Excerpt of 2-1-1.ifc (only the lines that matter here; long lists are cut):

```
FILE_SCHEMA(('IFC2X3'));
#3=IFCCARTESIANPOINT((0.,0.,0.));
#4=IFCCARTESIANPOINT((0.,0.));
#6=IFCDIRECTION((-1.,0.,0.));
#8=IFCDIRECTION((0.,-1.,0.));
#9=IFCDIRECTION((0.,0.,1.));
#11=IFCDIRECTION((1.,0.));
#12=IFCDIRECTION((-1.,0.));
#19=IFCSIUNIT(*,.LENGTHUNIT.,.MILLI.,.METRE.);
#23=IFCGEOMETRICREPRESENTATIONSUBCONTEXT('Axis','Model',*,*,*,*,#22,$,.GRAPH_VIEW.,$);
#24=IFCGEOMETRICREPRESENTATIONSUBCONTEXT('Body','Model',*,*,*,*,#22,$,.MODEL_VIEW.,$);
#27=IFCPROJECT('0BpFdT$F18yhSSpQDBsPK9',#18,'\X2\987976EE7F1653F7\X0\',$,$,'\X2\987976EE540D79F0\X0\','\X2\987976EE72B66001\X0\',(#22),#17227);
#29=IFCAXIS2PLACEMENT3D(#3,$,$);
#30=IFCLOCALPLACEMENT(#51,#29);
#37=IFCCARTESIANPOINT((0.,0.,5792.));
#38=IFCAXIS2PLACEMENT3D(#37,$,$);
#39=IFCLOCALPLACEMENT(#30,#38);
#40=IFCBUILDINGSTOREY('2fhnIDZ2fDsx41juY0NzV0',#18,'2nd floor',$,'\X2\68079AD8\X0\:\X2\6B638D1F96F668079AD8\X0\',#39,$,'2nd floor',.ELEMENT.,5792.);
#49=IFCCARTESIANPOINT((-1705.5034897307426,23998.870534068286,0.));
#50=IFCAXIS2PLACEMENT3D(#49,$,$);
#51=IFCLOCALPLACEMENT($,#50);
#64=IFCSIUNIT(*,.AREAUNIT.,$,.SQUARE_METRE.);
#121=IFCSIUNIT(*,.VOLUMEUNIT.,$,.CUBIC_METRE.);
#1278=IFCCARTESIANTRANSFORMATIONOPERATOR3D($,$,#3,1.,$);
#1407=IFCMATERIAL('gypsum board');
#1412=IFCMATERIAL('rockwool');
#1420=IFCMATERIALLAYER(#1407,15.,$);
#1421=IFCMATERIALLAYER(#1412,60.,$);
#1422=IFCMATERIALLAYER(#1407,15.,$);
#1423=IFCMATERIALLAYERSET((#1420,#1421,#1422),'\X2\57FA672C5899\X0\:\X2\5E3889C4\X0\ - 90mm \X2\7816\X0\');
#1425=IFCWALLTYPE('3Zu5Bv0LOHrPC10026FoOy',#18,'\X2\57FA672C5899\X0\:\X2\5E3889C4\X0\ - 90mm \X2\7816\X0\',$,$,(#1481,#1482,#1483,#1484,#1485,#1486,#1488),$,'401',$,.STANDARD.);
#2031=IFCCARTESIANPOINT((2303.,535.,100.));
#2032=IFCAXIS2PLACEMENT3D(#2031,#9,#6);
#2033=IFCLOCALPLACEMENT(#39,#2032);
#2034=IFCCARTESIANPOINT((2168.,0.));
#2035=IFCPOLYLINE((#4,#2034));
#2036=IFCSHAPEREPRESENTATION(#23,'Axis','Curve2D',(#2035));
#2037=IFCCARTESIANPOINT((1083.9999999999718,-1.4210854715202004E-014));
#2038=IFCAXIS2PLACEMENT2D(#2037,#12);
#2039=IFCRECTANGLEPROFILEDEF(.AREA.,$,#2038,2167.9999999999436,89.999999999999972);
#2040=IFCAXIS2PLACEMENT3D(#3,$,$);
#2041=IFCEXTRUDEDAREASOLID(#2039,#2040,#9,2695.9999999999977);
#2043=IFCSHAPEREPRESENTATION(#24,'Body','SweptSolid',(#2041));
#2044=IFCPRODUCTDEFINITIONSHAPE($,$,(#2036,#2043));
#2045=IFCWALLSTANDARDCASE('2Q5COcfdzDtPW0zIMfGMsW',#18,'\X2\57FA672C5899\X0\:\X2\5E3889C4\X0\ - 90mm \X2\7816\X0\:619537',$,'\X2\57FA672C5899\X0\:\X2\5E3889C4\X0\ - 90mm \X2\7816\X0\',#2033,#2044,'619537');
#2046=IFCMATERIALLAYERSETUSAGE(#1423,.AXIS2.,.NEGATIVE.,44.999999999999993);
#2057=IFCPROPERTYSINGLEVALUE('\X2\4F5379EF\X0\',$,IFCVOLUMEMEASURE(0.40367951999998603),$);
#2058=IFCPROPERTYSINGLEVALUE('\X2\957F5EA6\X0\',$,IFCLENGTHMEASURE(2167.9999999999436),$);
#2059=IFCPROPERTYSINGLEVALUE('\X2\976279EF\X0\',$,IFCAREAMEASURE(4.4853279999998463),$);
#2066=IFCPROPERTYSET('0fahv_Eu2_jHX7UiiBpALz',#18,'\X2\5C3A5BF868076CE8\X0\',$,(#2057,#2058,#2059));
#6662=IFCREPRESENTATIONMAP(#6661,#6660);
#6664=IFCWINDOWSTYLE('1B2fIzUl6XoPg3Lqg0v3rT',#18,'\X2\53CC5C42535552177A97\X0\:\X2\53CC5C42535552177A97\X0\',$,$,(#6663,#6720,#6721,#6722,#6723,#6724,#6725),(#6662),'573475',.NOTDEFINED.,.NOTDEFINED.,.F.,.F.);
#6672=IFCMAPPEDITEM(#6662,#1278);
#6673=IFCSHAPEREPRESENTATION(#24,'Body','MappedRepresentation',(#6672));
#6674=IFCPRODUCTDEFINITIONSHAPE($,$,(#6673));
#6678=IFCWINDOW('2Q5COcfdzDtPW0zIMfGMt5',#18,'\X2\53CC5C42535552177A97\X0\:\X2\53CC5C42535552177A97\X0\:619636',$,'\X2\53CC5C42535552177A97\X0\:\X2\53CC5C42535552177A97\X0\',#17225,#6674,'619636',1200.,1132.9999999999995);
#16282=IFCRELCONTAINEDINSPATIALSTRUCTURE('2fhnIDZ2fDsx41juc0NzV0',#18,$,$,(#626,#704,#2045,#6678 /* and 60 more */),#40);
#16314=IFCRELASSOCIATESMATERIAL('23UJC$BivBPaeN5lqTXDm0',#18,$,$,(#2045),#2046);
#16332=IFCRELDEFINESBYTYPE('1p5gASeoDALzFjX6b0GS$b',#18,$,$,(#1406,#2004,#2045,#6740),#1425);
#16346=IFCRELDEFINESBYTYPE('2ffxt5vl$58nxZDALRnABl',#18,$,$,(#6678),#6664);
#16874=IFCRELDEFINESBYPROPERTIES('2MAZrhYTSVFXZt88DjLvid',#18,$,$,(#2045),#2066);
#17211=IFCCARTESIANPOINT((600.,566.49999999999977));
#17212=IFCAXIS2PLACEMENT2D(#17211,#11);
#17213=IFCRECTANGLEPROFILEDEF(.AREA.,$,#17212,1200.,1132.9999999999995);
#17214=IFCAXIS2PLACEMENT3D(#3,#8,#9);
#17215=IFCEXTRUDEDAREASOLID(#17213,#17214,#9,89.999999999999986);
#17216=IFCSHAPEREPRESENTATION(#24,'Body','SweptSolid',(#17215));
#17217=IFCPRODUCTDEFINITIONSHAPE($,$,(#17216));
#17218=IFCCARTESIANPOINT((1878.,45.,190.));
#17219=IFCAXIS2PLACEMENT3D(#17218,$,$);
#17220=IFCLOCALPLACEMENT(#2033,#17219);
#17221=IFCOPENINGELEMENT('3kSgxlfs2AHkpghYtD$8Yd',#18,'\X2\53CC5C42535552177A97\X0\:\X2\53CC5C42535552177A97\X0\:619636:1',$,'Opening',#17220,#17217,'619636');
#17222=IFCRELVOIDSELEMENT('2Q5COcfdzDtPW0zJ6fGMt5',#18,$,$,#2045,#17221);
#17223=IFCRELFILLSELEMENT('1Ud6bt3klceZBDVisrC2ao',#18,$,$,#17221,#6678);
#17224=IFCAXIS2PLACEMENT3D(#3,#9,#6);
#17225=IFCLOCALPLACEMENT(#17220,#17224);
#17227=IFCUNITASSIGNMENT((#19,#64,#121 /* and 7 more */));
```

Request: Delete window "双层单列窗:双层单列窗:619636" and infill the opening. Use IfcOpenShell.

```python
import ifcopenshell
import ifcopenshell.api.feature
import ifcopenshell.api.pset
import ifcopenshell.api.root
import ifcopenshell.geom
import ifcopenshell.util.element
import ifcopenshell.util.shape
import ifcopenshell.util.unit

model = ifcopenshell.open("2-1-1.ifc")
area_scale = ifcopenshell.util.unit.calculate_unit_scale(model, "AREAUNIT")
volume_scale = ifcopenshell.util.unit.calculate_unit_scale(model, "VOLUMEUNIT")
settings = ifcopenshell.geom.settings()


def volume(element):
    """Net volume in cubic metres, openings subtracted."""
    shape = ifcopenshell.geom.create_shape(settings, element)
    return ifcopenshell.util.shape.get_volume(shape.geometry)


window = model.by_guid("2Q5COcfdzDtPW0zIMfGMt5")
opening = window.FillsVoids[0].RelatingOpeningElement
wall = opening.VoidsElements[0].RelatingBuildingElement
before = volume(wall)

ifcopenshell.api.root.remove_product(model, product=window)
ifcopenshell.api.feature.remove_feature(model, feature=opening)

after = volume(wall)
thickness = 0.09  # wall thickness in metres

# Update the wall's stored quantities.
pset = model.by_id(ifcopenshell.util.element.get_pset(wall, "尺寸标注", should_inherit=False)["id"])
ifcopenshell.api.pset.edit_pset(model, pset=pset, properties={
    "体积": model.create_entity("IfcVolumeMeasure", after / volume_scale),
    "面积": model.create_entity("IfcAreaMeasure", after / thickness / area_scale),
})

print(f"wall volume {before:.3f} -> {after:.3f} m3")

model.write("2-1-1-out.ifc")
```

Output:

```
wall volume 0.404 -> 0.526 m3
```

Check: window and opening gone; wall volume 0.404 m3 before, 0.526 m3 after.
